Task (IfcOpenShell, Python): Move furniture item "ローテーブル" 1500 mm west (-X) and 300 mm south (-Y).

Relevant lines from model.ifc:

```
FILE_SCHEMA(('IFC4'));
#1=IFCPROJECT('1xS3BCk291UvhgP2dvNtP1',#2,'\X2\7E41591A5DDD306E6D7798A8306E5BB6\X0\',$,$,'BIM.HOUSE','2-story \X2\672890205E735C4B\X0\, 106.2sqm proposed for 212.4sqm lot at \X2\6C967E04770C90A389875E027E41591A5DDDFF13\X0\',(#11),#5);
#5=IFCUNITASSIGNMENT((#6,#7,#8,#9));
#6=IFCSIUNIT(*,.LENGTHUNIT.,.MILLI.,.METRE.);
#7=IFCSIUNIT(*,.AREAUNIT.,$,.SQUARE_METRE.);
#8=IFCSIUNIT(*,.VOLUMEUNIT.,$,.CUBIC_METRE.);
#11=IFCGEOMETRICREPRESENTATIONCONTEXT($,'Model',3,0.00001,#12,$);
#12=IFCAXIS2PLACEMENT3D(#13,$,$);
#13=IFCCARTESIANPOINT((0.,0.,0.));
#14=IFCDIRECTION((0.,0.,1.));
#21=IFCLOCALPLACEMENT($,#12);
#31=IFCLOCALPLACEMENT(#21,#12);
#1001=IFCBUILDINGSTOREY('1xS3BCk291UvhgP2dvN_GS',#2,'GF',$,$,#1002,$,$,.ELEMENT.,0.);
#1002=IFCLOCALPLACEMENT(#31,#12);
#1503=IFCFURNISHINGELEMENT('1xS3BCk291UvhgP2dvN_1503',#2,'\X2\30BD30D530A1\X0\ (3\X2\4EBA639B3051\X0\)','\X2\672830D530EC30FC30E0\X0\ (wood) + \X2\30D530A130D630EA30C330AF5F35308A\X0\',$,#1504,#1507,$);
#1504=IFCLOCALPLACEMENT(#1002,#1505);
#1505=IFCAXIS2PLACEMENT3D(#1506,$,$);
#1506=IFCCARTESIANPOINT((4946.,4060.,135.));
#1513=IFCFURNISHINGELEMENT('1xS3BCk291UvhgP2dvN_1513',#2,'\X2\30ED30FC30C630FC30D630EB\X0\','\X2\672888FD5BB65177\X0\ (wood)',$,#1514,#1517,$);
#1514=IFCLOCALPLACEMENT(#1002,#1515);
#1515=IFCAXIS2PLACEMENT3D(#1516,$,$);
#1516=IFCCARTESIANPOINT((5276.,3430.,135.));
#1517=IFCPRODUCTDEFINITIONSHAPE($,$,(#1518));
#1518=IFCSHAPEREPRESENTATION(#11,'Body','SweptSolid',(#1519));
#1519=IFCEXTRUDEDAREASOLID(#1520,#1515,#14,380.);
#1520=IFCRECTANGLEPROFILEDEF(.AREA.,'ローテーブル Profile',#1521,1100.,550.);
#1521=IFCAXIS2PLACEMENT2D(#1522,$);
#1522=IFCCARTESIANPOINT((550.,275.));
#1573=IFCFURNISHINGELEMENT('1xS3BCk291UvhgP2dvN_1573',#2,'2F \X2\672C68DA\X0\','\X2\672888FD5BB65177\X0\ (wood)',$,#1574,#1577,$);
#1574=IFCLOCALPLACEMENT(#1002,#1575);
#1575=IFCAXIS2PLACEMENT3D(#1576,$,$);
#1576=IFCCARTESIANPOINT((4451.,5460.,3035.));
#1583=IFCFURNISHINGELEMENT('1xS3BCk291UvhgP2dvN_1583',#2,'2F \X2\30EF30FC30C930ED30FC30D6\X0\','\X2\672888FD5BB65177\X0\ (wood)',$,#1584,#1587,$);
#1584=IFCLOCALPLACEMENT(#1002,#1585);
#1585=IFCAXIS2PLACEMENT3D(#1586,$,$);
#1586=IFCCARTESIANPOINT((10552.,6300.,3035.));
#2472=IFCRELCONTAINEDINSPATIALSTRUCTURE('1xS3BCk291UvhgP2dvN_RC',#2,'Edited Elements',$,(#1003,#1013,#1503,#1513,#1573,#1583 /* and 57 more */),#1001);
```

```python
import ifcopenshell
import ifcopenshell.api.geometry
import ifcopenshell.util.placement
import ifcopenshell.util.unit

model = ifcopenshell.open("model.ifc")
unit_scale = ifcopenshell.util.unit.calculate_unit_scale(model)

item = model.by_id(1513)
matrix = ifcopenshell.util.placement.get_local_placement(item.ObjectPlacement)
matrix[0, 3] -= 1.5 / unit_scale
matrix[1, 3] -= 0.3 / unit_scale
ifcopenshell.api.geometry.edit_object_placement(model, product=item, matrix=matrix, is_si=False)

print(ifcopenshell.util.placement.get_local_placement(item.ObjectPlacement).round(3) + 0.0)

model.write("model_updated.ifc")
```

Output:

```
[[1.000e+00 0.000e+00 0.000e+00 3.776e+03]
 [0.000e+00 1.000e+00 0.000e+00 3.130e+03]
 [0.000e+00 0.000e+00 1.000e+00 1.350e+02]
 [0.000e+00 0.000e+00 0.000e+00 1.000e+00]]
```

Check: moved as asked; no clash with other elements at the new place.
